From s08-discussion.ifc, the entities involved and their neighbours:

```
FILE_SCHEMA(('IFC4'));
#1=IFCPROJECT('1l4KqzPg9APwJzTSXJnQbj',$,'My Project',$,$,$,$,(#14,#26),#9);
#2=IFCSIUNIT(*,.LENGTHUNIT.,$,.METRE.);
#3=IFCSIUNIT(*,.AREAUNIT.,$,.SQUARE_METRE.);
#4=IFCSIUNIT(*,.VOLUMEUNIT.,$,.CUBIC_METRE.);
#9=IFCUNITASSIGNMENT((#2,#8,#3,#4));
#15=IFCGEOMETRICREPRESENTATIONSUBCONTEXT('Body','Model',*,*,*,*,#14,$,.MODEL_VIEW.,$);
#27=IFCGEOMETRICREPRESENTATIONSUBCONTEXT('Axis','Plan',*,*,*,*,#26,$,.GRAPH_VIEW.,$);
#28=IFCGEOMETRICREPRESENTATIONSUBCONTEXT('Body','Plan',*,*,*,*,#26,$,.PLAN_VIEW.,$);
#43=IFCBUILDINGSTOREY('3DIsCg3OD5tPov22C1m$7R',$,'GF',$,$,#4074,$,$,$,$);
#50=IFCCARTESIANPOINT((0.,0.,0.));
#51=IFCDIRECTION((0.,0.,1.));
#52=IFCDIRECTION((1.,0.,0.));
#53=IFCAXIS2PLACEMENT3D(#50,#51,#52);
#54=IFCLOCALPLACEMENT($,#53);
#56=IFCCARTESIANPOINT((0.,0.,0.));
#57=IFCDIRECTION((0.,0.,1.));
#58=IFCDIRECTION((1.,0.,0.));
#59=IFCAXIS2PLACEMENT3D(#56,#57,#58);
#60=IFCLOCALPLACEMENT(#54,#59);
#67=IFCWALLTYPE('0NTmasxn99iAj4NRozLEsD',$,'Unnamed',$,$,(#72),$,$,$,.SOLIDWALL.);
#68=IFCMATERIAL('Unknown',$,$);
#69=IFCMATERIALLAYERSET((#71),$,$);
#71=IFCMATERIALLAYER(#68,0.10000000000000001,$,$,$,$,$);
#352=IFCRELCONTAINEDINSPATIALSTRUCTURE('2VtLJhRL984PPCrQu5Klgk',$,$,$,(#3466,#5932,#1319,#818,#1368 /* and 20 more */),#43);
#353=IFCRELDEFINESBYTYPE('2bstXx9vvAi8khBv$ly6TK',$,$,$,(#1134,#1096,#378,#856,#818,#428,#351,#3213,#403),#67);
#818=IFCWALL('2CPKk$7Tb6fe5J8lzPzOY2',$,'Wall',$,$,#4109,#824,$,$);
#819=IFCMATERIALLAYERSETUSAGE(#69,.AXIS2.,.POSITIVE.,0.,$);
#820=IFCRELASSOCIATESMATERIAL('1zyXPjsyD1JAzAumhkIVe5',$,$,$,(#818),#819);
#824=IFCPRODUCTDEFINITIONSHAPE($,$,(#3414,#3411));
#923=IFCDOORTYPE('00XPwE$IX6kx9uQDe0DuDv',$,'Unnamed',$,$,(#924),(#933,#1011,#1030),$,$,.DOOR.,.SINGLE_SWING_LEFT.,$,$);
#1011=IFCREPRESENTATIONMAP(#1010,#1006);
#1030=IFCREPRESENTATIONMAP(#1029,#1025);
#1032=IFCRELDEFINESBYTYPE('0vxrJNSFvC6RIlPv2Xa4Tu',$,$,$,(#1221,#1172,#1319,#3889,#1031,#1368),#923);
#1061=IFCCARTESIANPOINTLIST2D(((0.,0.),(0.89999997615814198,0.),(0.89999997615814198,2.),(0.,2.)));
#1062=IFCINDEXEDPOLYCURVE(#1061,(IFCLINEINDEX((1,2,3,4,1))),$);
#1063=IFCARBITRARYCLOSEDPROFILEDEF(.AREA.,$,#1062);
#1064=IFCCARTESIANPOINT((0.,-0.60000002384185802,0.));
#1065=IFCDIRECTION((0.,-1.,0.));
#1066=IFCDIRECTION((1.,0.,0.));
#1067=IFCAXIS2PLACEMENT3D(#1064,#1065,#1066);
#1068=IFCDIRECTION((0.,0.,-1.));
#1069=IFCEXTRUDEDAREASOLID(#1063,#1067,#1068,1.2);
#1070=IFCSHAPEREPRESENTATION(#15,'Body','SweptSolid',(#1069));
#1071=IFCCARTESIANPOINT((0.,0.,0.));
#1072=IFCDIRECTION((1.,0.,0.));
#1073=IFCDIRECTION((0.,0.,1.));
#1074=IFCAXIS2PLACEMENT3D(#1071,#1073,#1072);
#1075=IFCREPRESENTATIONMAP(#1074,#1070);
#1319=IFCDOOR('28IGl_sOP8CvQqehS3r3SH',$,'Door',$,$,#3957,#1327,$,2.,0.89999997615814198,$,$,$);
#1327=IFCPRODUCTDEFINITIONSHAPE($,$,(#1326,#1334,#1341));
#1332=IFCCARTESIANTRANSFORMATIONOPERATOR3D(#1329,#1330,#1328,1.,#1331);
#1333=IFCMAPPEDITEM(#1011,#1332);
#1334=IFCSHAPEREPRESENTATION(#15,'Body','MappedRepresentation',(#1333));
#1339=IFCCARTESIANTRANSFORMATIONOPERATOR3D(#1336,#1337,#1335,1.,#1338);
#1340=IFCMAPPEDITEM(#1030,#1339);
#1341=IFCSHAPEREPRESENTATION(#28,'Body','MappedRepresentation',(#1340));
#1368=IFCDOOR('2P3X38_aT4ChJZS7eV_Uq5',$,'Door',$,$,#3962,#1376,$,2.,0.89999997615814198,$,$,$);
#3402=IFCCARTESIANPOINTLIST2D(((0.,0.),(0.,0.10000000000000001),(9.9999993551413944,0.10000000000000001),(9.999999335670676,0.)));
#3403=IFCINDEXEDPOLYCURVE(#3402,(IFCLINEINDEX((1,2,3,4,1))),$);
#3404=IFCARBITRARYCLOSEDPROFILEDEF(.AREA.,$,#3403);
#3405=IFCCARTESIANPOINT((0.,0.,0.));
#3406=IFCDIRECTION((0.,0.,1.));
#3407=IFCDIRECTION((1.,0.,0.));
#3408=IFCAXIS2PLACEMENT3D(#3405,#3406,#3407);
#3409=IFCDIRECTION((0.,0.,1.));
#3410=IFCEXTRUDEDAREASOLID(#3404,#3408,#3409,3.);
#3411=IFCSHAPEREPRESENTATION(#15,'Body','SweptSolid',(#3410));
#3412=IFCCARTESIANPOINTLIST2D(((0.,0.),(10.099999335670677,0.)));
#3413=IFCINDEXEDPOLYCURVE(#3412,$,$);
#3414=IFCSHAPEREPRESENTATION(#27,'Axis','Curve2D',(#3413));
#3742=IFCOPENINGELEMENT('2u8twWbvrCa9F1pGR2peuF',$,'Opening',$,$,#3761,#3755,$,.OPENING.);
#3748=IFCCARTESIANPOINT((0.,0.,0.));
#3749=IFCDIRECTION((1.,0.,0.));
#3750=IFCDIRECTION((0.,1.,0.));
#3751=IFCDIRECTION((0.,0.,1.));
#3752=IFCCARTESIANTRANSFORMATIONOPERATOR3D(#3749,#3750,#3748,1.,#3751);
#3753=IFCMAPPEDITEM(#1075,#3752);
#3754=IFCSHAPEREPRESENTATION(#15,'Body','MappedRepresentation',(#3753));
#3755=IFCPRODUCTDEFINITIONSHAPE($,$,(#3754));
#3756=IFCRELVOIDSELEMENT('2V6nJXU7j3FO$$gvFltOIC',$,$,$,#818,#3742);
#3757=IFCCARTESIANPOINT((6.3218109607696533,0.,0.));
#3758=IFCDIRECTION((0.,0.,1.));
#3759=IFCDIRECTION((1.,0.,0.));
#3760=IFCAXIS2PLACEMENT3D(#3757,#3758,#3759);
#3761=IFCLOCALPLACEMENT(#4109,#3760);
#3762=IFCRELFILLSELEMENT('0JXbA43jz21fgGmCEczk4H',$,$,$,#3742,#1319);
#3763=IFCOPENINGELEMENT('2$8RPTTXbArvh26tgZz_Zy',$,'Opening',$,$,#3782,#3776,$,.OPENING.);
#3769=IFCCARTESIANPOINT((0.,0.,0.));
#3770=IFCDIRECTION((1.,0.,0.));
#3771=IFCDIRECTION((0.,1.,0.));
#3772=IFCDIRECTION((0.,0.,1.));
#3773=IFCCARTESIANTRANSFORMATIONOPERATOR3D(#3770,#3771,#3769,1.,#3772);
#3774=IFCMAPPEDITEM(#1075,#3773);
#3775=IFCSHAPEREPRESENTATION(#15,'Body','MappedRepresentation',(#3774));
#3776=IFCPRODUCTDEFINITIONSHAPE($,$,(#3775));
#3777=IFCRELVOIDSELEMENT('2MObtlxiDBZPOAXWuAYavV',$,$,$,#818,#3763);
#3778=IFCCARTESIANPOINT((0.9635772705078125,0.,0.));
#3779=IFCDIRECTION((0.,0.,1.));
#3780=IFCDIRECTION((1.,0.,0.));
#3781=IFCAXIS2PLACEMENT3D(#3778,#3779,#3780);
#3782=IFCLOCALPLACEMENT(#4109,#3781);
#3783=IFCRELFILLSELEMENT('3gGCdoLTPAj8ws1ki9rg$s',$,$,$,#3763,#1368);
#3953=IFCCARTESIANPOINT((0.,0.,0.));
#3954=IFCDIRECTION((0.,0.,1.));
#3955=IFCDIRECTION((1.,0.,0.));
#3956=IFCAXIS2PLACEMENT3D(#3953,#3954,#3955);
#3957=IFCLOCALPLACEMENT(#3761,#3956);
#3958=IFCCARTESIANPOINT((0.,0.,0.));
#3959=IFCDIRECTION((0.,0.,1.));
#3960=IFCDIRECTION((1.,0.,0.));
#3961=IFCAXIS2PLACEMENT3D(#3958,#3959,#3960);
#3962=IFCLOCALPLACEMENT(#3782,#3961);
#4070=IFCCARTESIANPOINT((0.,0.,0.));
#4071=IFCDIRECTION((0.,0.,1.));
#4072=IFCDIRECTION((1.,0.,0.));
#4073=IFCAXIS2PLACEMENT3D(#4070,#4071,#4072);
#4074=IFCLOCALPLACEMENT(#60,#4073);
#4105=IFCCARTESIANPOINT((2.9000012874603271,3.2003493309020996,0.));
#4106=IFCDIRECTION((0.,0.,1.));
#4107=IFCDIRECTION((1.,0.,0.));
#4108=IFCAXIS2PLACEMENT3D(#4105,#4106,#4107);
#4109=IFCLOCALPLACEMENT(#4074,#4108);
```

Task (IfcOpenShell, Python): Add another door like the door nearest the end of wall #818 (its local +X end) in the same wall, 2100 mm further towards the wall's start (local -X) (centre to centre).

```python
import ifcopenshell
import ifcopenshell.api.feature
import ifcopenshell.api.geometry
import ifcopenshell.api.root
import ifcopenshell.geom
import ifcopenshell.util.element
import ifcopenshell.util.placement
import ifcopenshell.util.shape
import ifcopenshell.util.unit

model = ifcopenshell.open("s08-discussion.ifc")
unit_scale = ifcopenshell.util.unit.calculate_unit_scale(model)
settings = ifcopenshell.geom.settings()


def volume(element):
    """Net volume in cubic metres, openings subtracted."""
    shape = ifcopenshell.geom.create_shape(settings, element)
    return ifcopenshell.util.shape.get_volume(shape.geometry)


door = model.by_guid("28IGl_sOP8CvQqehS3r3SH")
opening = door.FillsVoids[0].RelatingOpeningElement
wall = opening.VoidsElements[0].RelatingBuildingElement
before = volume(wall)
shift = ifcopenshell.util.placement.get_local_placement(wall.ObjectPlacement)[:3, 0] * -2.1 / unit_scale

# copy_class copies the void relationship, type, container and properties, but no geometry.
new_opening = ifcopenshell.api.root.copy_class(model, product=opening)
new_opening.Representation = ifcopenshell.util.element.copy_deep(
    model, opening.Representation, exclude=["IfcGeometricRepresentationContext", "IfcRepresentationMap"]
)
new_door = ifcopenshell.api.root.copy_class(model, product=door)
new_door.Representation = ifcopenshell.util.element.copy_deep(
    model, door.Representation, exclude=["IfcGeometricRepresentationContext", "IfcRepresentationMap"]
)
ifcopenshell.api.feature.add_filling(model, opening=new_opening, element=new_door)

for old, new in ((opening, new_opening), (door, new_door)):
    matrix = ifcopenshell.util.placement.get_local_placement(old.ObjectPlacement)
    matrix[:3, 3] += shift
    ifcopenshell.api.geometry.edit_object_placement(model, product=new, matrix=matrix, is_si=False)

after = volume(wall)

print(f"wall volume {before:.3f} -> {after:.3f} m3")

model.write("s08-discussion-out.ifc")
```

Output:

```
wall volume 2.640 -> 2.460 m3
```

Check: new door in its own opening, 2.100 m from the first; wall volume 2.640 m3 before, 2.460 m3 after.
